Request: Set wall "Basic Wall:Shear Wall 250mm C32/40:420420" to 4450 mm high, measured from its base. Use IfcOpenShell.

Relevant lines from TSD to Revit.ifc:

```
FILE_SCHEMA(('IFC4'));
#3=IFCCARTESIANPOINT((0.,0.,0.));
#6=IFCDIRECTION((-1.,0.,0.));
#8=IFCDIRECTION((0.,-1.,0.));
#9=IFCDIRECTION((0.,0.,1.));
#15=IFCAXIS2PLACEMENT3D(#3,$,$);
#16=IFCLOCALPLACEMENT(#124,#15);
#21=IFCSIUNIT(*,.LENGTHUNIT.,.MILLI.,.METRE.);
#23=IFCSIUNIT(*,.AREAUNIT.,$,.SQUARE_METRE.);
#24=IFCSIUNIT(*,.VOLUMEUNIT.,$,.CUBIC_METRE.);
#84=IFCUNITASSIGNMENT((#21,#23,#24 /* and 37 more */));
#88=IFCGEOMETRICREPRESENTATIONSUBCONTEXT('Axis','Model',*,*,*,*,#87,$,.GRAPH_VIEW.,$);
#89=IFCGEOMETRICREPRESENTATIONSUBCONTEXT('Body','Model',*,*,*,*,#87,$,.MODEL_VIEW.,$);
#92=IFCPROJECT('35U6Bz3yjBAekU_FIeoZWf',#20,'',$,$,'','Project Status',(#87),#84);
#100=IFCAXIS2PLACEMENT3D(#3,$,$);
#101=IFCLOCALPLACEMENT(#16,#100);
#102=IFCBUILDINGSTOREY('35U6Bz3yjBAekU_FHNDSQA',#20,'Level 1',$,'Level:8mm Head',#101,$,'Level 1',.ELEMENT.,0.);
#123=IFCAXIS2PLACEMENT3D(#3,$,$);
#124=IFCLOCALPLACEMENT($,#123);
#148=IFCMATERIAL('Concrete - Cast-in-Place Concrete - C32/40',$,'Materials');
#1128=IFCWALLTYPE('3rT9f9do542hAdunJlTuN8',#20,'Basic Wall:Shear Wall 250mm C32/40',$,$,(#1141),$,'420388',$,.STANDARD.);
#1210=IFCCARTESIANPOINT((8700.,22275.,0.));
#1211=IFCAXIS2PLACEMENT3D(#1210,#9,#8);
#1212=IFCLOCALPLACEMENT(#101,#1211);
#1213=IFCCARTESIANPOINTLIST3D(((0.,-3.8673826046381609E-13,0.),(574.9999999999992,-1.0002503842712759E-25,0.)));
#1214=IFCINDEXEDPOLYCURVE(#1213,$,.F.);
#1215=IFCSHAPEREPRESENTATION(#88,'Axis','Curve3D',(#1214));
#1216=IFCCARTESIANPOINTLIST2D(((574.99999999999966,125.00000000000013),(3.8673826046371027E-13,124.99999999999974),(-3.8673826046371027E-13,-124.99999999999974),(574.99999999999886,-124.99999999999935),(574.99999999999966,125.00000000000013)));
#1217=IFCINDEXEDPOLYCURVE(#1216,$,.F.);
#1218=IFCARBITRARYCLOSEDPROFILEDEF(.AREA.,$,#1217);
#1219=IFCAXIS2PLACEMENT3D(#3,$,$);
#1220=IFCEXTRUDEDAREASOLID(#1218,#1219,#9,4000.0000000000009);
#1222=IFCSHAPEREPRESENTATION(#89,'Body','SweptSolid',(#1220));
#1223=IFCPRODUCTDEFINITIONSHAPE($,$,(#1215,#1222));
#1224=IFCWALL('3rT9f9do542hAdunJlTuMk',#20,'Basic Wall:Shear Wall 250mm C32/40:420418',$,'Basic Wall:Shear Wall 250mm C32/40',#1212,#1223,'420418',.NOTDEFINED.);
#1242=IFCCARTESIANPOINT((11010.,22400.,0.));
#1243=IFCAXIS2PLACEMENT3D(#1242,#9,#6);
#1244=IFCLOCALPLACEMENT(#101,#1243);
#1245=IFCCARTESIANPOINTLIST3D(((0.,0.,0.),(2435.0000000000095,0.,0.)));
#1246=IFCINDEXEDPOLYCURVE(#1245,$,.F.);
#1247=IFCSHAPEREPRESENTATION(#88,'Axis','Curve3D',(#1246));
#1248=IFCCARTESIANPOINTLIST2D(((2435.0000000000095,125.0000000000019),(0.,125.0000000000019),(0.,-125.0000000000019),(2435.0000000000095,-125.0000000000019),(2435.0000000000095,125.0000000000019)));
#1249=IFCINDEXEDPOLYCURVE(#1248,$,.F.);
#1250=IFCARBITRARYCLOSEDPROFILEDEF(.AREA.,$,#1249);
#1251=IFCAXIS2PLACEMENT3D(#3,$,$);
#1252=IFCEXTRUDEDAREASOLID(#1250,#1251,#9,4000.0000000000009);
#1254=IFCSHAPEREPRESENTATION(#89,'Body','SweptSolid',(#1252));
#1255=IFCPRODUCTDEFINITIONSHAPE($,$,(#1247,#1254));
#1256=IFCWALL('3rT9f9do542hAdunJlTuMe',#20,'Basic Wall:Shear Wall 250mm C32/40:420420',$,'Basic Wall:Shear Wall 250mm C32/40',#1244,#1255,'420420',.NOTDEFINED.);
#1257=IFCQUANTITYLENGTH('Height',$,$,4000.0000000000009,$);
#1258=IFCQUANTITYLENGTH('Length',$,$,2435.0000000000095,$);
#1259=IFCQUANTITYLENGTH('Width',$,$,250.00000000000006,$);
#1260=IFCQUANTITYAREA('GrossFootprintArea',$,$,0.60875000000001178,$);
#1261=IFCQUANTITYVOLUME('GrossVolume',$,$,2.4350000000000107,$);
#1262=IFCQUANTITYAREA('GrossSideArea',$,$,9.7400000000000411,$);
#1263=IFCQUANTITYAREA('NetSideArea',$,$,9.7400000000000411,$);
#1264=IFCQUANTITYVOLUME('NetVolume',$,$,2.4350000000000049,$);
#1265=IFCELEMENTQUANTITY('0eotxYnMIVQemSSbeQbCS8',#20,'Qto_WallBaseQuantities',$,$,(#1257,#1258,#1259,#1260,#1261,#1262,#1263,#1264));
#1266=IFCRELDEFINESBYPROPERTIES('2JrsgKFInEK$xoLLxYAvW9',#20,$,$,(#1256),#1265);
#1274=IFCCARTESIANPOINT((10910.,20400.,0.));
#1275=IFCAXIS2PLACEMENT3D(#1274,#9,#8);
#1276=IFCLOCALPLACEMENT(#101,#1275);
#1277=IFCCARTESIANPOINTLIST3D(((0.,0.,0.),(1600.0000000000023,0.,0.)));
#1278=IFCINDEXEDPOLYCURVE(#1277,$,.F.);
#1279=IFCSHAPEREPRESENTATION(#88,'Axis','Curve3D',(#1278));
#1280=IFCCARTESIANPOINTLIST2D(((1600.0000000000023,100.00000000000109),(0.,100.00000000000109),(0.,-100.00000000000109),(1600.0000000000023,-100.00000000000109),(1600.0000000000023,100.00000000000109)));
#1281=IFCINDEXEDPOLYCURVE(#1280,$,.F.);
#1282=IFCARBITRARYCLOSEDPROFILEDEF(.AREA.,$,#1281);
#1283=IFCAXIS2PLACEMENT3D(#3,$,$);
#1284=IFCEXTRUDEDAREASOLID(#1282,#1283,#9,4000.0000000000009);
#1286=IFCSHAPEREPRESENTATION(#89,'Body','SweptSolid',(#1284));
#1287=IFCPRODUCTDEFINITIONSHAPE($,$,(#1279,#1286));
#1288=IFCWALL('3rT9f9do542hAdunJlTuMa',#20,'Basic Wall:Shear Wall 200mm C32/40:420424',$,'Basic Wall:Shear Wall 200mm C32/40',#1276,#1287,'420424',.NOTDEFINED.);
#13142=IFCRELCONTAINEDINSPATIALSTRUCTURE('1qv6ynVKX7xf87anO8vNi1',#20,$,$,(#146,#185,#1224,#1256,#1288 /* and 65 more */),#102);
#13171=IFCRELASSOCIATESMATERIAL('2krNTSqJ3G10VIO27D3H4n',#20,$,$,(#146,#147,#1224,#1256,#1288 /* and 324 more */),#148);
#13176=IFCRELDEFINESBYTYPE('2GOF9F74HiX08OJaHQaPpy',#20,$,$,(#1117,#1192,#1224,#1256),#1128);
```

```python
import ifcopenshell
import ifcopenshell.api.pset
import ifcopenshell.geom
import ifcopenshell.util.element
import ifcopenshell.util.representation
import ifcopenshell.util.shape
import ifcopenshell.util.unit

model = ifcopenshell.open("TSD to Revit.ifc")
unit_scale = ifcopenshell.util.unit.calculate_unit_scale(model)
area_scale = ifcopenshell.util.unit.calculate_unit_scale(model, "AREAUNIT")
volume_scale = ifcopenshell.util.unit.calculate_unit_scale(model, "VOLUMEUNIT")
settings = ifcopenshell.geom.settings()


def volume(element):
    """Net volume in cubic metres, openings subtracted."""
    shape = ifcopenshell.geom.create_shape(settings, element)
    return ifcopenshell.util.shape.get_volume(shape.geometry)


wall = model.by_guid("3rT9f9do542hAdunJlTuMe")
before = volume(wall)

body = ifcopenshell.util.representation.get_representation(wall, "Model", "Body")
solid = body.Items[0]
old_height = solid.Depth
solid.Depth = 4450.0
after = volume(wall)
thickness = 0.25  # wall thickness in metres

# Update the stored height, areas and volumes.
qto = model.by_id(ifcopenshell.util.element.get_pset(wall, "Qto_WallBaseQuantities", should_inherit=False)["id"])
ifcopenshell.api.pset.edit_qto(model, qto=qto, properties={
    "Height": solid.Depth,
    "GrossVolume": ifcopenshell.util.element.get_pset(wall, "Qto_WallBaseQuantities", "GrossVolume") * solid.Depth / old_height,
    "GrossSideArea": ifcopenshell.util.element.get_pset(wall, "Qto_WallBaseQuantities", "GrossSideArea") * solid.Depth / old_height,
    "NetSideArea": after / thickness / area_scale,
    "NetVolume": after / volume_scale,
})

print(f"height {old_height:g} -> {solid.Depth:g}, volume {before:.3f} -> {after:.3f} m3")

model.write("TSD to Revit_edited.ifc")
```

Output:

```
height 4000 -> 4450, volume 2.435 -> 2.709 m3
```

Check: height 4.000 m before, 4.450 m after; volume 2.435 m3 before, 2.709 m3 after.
